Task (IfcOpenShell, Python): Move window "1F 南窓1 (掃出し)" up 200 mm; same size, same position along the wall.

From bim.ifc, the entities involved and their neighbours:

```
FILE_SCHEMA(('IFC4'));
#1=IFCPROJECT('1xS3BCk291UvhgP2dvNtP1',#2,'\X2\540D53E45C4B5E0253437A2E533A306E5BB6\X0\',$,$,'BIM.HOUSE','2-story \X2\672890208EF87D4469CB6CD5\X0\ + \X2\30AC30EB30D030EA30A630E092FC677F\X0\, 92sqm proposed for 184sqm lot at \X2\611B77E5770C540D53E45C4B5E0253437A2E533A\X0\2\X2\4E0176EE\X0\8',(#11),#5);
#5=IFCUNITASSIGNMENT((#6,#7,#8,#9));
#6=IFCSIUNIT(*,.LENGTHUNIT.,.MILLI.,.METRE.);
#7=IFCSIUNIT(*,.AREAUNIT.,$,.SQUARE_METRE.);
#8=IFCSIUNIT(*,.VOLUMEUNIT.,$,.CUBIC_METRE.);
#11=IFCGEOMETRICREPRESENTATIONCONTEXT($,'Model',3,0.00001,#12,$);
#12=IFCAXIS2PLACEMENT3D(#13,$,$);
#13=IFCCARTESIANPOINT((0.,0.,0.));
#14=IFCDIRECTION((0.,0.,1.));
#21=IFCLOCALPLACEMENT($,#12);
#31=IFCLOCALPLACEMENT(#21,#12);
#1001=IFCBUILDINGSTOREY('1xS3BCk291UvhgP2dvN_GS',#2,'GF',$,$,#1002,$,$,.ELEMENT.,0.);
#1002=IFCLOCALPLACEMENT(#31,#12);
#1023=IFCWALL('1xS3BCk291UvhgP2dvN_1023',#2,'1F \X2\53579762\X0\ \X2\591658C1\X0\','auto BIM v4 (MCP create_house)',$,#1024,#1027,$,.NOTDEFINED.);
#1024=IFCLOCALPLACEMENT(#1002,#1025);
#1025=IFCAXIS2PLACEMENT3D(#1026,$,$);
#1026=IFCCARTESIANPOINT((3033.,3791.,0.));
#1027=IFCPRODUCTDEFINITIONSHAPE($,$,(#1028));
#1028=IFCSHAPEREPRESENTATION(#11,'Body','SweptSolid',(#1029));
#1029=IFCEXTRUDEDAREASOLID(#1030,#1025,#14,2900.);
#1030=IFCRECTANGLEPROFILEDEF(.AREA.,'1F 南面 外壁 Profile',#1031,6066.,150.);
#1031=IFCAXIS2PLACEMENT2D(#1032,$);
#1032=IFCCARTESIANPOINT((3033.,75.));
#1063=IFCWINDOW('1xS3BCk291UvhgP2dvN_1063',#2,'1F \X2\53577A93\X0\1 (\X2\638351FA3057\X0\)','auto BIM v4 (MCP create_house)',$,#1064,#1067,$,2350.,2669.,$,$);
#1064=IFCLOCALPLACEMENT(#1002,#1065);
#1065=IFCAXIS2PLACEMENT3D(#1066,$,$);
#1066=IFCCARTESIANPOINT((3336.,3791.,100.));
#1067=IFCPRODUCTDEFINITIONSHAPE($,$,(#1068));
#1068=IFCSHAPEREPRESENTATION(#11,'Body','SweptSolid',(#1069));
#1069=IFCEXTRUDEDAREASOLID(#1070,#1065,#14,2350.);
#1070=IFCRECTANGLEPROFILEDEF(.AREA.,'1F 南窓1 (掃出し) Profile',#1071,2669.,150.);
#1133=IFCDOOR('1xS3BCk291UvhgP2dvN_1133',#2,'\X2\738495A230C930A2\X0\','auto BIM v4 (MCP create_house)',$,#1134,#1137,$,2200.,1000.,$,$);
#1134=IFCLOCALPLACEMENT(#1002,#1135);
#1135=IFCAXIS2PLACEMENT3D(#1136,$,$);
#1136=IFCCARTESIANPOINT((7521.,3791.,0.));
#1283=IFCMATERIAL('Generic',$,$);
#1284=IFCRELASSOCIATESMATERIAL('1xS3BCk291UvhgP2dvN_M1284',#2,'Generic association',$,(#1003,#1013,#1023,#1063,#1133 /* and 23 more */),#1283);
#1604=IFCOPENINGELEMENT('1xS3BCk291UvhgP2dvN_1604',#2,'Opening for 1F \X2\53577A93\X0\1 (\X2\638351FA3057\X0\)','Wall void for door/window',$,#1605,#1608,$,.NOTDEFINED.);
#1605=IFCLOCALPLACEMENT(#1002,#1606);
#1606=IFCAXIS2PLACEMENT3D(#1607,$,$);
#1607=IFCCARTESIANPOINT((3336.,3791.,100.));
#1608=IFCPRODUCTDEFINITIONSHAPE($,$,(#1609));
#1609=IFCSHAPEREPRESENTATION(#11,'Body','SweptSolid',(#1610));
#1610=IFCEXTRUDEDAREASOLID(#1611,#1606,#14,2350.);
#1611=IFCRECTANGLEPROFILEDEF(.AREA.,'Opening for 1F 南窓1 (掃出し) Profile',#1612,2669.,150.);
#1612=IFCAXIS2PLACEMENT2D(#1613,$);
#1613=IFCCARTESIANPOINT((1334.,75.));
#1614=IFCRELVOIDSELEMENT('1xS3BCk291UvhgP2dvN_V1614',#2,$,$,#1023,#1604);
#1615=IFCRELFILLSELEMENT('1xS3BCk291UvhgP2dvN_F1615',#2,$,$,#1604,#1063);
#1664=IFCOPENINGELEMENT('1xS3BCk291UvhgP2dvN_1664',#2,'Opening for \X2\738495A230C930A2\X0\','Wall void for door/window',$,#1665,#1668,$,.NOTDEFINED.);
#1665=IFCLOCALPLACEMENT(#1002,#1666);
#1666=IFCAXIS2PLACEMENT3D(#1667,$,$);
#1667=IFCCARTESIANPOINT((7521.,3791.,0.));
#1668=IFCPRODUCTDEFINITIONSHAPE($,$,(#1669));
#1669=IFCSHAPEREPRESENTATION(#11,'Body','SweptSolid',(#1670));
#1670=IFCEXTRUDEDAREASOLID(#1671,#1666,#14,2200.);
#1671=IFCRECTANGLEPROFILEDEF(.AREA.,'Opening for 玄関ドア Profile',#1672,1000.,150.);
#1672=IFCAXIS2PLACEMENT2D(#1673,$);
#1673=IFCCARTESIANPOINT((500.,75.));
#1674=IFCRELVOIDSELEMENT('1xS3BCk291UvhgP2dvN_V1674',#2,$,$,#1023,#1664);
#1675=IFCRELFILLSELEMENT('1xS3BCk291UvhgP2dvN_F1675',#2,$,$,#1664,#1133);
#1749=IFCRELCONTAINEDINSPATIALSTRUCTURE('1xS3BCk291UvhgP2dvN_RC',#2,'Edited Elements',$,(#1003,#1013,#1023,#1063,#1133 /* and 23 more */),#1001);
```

```python
import numpy as np
import ifcopenshell
import ifcopenshell.api.geometry
import ifcopenshell.util.placement
import ifcopenshell.util.unit

model = ifcopenshell.open("bim.ifc")
unit_scale = ifcopenshell.util.unit.calculate_unit_scale(model)

window = model.by_id(1063)
opening = window.FillsVoids[0].RelatingOpeningElement
dz = 200.0

shift = np.array([0.0, 0.0, dz])
# The window is not placed relative to its opening, so move both.
for product in (opening, window):
    matrix = ifcopenshell.util.placement.get_local_placement(product.ObjectPlacement)
    matrix[:3, 3] += shift
    ifcopenshell.api.geometry.edit_object_placement(model, product=product, matrix=matrix, is_si=False)

print(f"moved by {dz * unit_scale:+.3f} m")

model.write("bim_v2.ifc")
```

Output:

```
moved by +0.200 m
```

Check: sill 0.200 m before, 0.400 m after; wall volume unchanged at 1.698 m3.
